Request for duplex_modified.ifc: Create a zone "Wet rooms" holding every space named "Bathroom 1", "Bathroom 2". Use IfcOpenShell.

First a look at what the model holds.

```python
import ifcopenshell

model = ifcopenshell.open("duplex_modified.ifc")
print(model.schema)
seen = {}
for space in model.by_type("IfcSpace"):
    seen[space.LongName] = seen.get(space.LongName, 0) + 1
for name, count in sorted(seen.items(), key=str):
    print(count, "x", name)
print("zones:", [z.Name for z in model.by_type("IfcZone")][:20])
```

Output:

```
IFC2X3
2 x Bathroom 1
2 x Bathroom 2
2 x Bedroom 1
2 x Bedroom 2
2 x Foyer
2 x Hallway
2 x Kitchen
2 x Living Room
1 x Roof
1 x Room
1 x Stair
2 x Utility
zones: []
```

```python
import ifcopenshell
import ifcopenshell.api.group
import ifcopenshell.api.root

model = ifcopenshell.open("duplex_modified.ifc")

names = {"Bathroom 1", "Bathroom 2"}
spaces = [s for s in model.by_type("IfcSpace") if s.LongName in names]

zone = ifcopenshell.api.root.create_entity(model, ifc_class="IfcZone", name="Wet rooms")
ifcopenshell.api.group.assign_group(model, products=spaces, group=zone)
print(len(spaces), "spaces in", zone.Name)

model.write("duplex_modified-out.ifc")
```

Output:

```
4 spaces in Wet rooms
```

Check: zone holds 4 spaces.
